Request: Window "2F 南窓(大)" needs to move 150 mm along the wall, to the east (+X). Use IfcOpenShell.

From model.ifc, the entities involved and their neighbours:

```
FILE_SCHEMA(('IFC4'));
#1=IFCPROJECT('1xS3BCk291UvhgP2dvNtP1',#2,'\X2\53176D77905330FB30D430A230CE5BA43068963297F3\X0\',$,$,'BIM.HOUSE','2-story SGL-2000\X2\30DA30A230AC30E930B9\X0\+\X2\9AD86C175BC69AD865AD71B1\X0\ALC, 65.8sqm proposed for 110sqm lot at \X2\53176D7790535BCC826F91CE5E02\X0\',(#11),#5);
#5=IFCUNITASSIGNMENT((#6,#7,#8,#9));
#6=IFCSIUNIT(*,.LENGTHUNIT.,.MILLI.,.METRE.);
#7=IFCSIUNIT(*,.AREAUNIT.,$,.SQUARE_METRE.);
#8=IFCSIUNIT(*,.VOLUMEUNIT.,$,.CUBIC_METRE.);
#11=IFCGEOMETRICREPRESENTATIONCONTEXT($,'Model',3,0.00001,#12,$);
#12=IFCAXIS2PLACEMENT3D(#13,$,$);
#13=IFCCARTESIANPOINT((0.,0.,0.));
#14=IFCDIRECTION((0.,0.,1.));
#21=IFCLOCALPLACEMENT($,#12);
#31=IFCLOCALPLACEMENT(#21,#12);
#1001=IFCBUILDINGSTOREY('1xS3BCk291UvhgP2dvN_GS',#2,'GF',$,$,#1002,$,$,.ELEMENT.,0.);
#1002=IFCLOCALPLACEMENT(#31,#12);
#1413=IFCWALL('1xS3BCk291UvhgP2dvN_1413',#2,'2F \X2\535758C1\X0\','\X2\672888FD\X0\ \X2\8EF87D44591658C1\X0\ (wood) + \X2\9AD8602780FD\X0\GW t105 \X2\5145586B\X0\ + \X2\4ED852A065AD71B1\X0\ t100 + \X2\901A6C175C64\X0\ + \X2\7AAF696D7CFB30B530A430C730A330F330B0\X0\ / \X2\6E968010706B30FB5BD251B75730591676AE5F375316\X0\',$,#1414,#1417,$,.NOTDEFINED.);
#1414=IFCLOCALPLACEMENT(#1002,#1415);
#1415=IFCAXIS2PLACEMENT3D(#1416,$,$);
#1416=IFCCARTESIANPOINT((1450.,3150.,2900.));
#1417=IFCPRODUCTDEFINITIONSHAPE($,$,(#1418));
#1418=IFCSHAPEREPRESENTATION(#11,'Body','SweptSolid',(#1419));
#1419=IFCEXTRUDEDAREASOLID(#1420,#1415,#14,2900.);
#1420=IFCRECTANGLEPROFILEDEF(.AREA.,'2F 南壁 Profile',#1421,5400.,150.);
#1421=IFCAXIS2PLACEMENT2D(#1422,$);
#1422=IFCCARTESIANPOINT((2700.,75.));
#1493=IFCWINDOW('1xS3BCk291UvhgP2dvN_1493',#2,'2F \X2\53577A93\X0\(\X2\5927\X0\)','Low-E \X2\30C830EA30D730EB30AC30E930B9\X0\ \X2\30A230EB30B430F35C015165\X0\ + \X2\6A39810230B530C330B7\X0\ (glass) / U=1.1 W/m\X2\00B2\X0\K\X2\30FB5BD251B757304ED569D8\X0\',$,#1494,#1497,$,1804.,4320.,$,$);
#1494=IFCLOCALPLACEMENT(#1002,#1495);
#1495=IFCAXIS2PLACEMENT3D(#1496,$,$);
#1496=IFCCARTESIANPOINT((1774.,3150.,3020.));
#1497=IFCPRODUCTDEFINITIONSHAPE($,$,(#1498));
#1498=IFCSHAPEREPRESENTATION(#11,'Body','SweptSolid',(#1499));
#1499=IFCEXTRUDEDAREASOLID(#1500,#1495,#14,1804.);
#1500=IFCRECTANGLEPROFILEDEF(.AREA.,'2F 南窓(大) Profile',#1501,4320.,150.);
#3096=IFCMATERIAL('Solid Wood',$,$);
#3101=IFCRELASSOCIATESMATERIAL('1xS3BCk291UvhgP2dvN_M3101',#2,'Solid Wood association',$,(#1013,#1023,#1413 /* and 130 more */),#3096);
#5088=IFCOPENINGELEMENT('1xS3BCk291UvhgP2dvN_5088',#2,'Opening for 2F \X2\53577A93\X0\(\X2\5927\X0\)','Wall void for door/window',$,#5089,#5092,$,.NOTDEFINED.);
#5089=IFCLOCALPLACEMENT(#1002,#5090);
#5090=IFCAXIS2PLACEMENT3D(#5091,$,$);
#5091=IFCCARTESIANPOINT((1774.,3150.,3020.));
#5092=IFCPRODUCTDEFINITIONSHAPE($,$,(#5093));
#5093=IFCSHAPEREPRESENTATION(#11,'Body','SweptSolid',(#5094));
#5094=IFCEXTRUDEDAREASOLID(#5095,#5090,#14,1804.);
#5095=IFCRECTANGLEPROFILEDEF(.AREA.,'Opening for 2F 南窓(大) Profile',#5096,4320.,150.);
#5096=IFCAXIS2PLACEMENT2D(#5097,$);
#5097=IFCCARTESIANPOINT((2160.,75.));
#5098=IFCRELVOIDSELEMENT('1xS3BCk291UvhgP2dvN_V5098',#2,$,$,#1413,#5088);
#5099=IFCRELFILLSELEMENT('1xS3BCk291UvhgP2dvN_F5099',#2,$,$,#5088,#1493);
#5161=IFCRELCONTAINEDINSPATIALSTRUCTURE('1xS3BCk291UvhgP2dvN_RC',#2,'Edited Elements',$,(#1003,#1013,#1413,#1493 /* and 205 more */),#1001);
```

```python
import ifcopenshell
import ifcopenshell.api.geometry
import ifcopenshell.util.placement
import ifcopenshell.util.unit

model = ifcopenshell.open("model.ifc")
unit_scale = ifcopenshell.util.unit.calculate_unit_scale(model)

window = model.by_guid("1xS3BCk291UvhgP2dvN_1493")
opening = window.FillsVoids[0].RelatingOpeningElement
wall = opening.VoidsElements[0].RelatingBuildingElement

wall_matrix = ifcopenshell.util.placement.get_local_placement(wall.ObjectPlacement)
shift = wall_matrix[:3, 0] * 0.15 / unit_scale
before = ifcopenshell.util.placement.get_local_placement(window.ObjectPlacement)[:3, 3].copy()

# The window is not placed relative to its opening, so move both.
for product in (opening, window):
    matrix = ifcopenshell.util.placement.get_local_placement(product.ObjectPlacement)
    matrix[:3, 3] += shift
    ifcopenshell.api.geometry.edit_object_placement(model, product=product, matrix=matrix, is_si=False)

after = ifcopenshell.util.placement.get_local_placement(window.ObjectPlacement)[:3, 3]
print("window moved by", (after - before).round(3) + 0.0)

model.write("model_v2.ifc")
```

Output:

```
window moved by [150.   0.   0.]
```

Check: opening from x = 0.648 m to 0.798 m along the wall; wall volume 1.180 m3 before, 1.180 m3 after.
